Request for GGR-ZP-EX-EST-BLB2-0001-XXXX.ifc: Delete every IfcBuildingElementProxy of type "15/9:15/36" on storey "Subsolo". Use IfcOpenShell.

First a look at what the model holds.

```python
import ifcopenshell
import ifcopenshell.util.element

model = ifcopenshell.open("GGR-ZP-EX-EST-BLB2-0001-XXXX.ifc")
print(model.schema)
storey = next(s for s in model.by_type("IfcBuildingStorey") if s.Name == "Subsolo")
proxies = [e for e in ifcopenshell.util.element.get_decomposition(storey) if e.is_a("IfcBuildingElementProxy")]
seen = {}
for e in proxies:
    element_type = ifcopenshell.util.element.get_type(e)
    name = element_type.Name if element_type not in (None, e) else None
    seen[name] = seen.get(name, 0) + 1
for name, count in sorted(seen.items(), key=str):
    print(count, "x", name)
```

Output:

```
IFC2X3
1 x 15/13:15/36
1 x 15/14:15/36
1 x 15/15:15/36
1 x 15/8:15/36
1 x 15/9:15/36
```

```python
import ifcopenshell
import ifcopenshell.api.root
import ifcopenshell.util.element

model = ifcopenshell.open("GGR-ZP-EX-EST-BLB2-0001-XXXX.ifc")

storey = next(s for s in model.by_type("IfcBuildingStorey") if s.Name == "Subsolo")
proxies = [e for e in ifcopenshell.util.element.get_decomposition(storey) if e.is_a("IfcBuildingElementProxy")]
targets = [e for e in proxies if (t := ifcopenshell.util.element.get_type(e)) not in (None, e) and t.Name == "15/9:15/36"]

for e in targets:
    ifcopenshell.api.root.remove_product(model, product=e)
print(len(targets), "removed")

model.write("GGR-ZP-EX-EST-BLB2-0001-XXXX_v2.ifc")
```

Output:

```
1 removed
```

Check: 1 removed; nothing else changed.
